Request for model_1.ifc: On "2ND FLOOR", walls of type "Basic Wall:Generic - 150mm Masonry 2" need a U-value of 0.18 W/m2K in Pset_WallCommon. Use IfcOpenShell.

First a look at what the model holds.

```python
import ifcopenshell
import ifcopenshell.util.element

model = ifcopenshell.open("model_1.ifc")
print(model.schema)
storey = next(s for s in model.by_type("IfcBuildingStorey") if s.Name == "2ND FLOOR")
walls = [e for e in ifcopenshell.util.element.get_decomposition(storey) if e.is_a("IfcWall")]
seen = {}
for e in walls:
    element_type = ifcopenshell.util.element.get_type(e)
    key = (element_type.Name if element_type != e and element_type else None, ifcopenshell.util.element.get_pset(e, "Pset_WallCommon", "ThermalTransmittance"))
    seen[key] = seen.get(key, 0) + 1
for (name, value), count in sorted(seen.items(), key=str):
    print(count, "x", name, "|", value)
```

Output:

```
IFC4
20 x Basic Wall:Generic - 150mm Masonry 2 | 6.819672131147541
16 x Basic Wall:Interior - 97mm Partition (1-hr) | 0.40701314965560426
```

```python
import ifcopenshell
import ifcopenshell.api.pset
import ifcopenshell.util.element

model = ifcopenshell.open("model_1.ifc")

storey = next(s for s in model.by_type("IfcBuildingStorey") if s.Name == "2ND FLOOR")
walls = [e for e in ifcopenshell.util.element.get_decomposition(storey) if e.is_a("IfcWall")]

count = 0
for e in walls:
    element_type = ifcopenshell.util.element.get_type(e)
    if element_type in (None, e) or element_type.Name != "Basic Wall:Generic - 150mm Masonry 2":
        continue
    # add_pset returns the element's existing set when there is one.
    pset = ifcopenshell.api.pset.add_pset(model, product=e, name="Pset_WallCommon")
    ifcopenshell.api.pset.edit_pset(model, pset=pset, properties={"ThermalTransmittance": 0.18})
    count += 1

print(count, "walls updated")

model.write("model_1_edited.ifc")
```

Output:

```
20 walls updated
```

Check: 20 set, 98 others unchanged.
